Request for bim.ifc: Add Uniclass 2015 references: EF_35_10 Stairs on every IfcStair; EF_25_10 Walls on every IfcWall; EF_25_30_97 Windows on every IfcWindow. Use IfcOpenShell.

First a look at what the model holds.

```python
import ifcopenshell

model = ifcopenshell.open("bim.ifc")
print(model.schema)
print("classifications:", [c.Name for c in model.by_type("IfcClassification")])
for ifc_class in ("IfcDoor", "IfcRoof", "IfcStair", "IfcWall", "IfcWindow"):
    print(ifc_class, len(model.by_type(ifc_class)))
```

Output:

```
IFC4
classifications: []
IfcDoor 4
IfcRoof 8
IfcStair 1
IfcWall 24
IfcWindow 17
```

```python
import ifcopenshell
import ifcopenshell.api.classification

model = ifcopenshell.open("bim.ifc")

system = ifcopenshell.api.classification.add_classification(model, classification="Uniclass 2015")

codes = {
    "IfcStair": ("EF_35_10", "Stairs"),
    "IfcWall": ("EF_25_10", "Walls"),
    "IfcWindow": ("EF_25_30_97", "Windows"),
}
for ifc_class, (code, name) in codes.items():
    products = model.by_type(ifc_class)
    ifcopenshell.api.classification.add_reference(
        model, products=products, classification=system, identification=code, name=name
    )
    print(code, len(products))

model.write("bim-out.ifc")
```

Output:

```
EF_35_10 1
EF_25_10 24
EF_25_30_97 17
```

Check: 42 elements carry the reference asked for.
